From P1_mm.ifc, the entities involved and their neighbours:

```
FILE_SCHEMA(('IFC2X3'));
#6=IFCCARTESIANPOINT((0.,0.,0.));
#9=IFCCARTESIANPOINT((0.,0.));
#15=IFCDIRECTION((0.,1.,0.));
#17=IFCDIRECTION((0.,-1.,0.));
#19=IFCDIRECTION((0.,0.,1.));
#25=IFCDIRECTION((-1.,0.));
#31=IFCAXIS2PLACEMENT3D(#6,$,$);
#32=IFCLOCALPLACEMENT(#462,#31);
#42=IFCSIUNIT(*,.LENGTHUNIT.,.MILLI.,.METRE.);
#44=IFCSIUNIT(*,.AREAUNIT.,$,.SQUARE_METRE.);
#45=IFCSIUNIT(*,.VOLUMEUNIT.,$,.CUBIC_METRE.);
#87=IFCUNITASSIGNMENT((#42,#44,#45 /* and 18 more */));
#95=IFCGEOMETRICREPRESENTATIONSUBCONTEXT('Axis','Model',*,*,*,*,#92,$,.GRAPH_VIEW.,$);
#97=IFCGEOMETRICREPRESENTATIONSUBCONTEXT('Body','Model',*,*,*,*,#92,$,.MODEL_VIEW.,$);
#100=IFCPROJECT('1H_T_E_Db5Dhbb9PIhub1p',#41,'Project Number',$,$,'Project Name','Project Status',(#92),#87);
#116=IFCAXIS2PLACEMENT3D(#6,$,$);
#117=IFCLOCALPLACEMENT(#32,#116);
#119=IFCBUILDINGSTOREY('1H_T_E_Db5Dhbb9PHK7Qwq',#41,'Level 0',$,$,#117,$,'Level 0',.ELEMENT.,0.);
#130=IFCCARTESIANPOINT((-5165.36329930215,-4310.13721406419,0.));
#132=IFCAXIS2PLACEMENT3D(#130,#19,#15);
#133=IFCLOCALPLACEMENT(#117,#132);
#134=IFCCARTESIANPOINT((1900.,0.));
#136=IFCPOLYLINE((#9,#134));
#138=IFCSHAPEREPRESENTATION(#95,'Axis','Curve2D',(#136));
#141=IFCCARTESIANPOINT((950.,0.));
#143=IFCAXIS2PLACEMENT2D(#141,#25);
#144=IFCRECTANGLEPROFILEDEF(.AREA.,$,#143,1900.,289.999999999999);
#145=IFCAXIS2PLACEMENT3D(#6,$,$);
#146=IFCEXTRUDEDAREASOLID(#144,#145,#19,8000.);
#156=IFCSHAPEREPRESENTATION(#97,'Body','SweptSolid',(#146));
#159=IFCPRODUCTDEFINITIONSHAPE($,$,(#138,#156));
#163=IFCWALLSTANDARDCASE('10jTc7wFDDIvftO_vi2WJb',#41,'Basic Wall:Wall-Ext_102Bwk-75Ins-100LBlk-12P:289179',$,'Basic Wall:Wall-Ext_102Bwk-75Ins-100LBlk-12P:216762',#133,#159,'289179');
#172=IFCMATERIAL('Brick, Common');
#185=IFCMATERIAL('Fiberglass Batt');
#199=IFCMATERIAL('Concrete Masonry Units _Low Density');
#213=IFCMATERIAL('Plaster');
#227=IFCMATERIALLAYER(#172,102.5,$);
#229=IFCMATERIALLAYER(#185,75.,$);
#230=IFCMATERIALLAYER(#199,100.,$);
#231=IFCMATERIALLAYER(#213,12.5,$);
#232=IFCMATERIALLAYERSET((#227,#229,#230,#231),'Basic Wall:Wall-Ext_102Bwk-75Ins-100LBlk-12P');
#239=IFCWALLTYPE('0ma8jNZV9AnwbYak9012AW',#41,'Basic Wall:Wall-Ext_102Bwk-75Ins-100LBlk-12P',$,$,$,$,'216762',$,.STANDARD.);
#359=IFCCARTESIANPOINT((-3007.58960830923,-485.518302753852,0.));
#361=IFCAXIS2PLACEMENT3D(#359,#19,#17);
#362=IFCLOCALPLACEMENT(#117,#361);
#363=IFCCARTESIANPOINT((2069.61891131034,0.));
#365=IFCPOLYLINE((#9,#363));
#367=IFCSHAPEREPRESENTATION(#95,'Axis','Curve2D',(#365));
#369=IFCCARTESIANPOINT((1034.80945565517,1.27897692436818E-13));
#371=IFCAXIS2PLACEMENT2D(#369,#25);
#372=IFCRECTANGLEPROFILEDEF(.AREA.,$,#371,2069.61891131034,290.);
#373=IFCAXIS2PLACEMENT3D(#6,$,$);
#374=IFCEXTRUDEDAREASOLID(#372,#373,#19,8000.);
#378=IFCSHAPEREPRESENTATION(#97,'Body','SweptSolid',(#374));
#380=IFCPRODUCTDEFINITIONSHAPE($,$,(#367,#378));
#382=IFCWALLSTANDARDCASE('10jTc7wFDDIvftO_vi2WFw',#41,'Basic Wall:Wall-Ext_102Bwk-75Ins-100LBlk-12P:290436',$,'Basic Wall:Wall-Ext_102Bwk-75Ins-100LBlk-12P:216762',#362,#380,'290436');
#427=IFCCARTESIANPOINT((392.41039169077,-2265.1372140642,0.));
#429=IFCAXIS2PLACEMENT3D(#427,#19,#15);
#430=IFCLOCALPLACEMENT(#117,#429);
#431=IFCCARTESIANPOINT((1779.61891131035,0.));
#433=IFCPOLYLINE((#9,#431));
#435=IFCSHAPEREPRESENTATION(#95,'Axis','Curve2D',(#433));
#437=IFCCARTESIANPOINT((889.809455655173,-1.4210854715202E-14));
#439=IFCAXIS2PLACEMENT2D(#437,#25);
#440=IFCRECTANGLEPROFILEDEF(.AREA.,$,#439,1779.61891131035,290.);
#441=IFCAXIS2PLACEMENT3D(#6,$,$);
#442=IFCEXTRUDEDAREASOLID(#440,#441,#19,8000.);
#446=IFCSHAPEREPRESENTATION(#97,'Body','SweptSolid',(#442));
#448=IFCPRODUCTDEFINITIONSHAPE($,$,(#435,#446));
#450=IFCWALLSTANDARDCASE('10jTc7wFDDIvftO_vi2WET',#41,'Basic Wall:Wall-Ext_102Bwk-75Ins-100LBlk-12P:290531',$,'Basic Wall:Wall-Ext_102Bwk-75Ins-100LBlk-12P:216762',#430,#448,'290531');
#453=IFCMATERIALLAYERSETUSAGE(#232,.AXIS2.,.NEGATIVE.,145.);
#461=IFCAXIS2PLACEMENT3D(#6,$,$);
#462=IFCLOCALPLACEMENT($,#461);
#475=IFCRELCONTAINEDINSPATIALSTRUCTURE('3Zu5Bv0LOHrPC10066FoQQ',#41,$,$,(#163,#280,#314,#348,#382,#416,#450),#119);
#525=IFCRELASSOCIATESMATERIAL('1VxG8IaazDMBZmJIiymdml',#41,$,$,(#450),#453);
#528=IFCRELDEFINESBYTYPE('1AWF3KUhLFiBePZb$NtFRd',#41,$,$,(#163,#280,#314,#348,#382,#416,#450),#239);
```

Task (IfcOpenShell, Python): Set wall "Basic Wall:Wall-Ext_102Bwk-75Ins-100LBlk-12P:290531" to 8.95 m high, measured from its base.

```python
import ifcopenshell
import ifcopenshell.geom
import ifcopenshell.util.representation
import ifcopenshell.util.shape

model = ifcopenshell.open("P1_mm.ifc")
settings = ifcopenshell.geom.settings()


def volume(element):
    """Net volume in cubic metres, openings subtracted."""
    shape = ifcopenshell.geom.create_shape(settings, element)
    return ifcopenshell.util.shape.get_volume(shape.geometry)


wall = model.by_id(450)
before = volume(wall)

body = ifcopenshell.util.representation.get_representation(wall, "Model", "Body")
solid = body.Items[0]
old_height = solid.Depth
solid.Depth = 8950.0
after = volume(wall)

print(f"height {old_height:g} -> {solid.Depth:g}, volume {before:.3f} -> {after:.3f} m3")

model.write("P1_mm-out.ifc")
```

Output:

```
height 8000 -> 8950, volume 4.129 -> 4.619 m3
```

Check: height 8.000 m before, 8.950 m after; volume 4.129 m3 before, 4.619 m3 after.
